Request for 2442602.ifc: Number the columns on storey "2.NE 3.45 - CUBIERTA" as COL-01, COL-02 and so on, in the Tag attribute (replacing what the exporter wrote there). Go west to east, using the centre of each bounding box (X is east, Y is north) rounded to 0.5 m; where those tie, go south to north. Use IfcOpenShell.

First a look at what the model holds.

```python
import ifcopenshell
import ifcopenshell.util.element
import ifcopenshell.util.placement

model = ifcopenshell.open("2442602.ifc")
print(model.schema)
storey = next(s for s in model.by_type("IfcBuildingStorey") if s.Name == "2.NE 3.45 - CUBIERTA")
columns = [e for e in ifcopenshell.util.element.get_decomposition(storey) if e.is_a("IfcColumn")]
for e in sorted(columns, key=lambda e: e.id()):
    origin = ifcopenshell.util.placement.get_local_placement(e.ObjectPlacement)[:3, 3]
    print(e.id(), e.Tag, e.Name, origin.round(2) + 0.0, sep=" | ")
```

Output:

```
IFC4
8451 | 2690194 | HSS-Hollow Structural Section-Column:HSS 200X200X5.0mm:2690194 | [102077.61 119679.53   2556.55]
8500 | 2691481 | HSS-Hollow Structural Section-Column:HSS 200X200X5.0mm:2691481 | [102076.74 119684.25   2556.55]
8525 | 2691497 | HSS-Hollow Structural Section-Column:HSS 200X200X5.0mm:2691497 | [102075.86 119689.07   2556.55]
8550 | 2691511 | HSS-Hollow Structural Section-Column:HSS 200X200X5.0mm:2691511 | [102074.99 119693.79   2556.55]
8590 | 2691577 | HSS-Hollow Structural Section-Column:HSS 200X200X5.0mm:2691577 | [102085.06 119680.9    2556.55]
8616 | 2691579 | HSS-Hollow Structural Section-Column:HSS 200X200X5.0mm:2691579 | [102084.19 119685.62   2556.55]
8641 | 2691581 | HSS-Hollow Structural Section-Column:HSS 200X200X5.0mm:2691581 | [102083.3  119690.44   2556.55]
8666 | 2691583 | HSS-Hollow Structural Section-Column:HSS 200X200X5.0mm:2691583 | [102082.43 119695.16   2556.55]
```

```python
import ifcopenshell
import ifcopenshell.geom
import ifcopenshell.util.element
import ifcopenshell.util.shape

model = ifcopenshell.open("2442602.ifc")
settings = ifcopenshell.geom.settings()
settings.set("use-world-coords", True)


def centre(element):
    shape = ifcopenshell.geom.create_shape(settings, element)
    return ifcopenshell.util.shape.get_bbox_centroid(shape.geometry)


storey = next(s for s in model.by_type("IfcBuildingStorey") if s.Name == "2.NE 3.45 - CUBIERTA")
columns = [e for e in ifcopenshell.util.element.get_decomposition(storey) if e.is_a("IfcColumn")]

# Insertion points can sit at a corner or the storey origin, so sort by the geometry (in metres).
centres = {e: centre(e) for e in columns}
columns.sort(key=lambda e: (round(centres[e][0] / 0.5), centres[e][1]))

for i, e in enumerate(columns, start=1):
    number = f"COL-{i:02d}"
    e.Tag = number
    print(e.id(), number)

model.write("2442602_updated.ifc")
```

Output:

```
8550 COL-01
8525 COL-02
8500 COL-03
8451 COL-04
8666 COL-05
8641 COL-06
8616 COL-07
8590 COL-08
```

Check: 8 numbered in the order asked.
